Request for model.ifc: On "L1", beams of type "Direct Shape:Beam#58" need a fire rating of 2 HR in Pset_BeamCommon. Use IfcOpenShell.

First a look at what the model holds.

```python
import ifcopenshell
import ifcopenshell.util.element

model = ifcopenshell.open("model.ifc")
print(model.schema)
storey = next(s for s in model.by_type("IfcBuildingStorey") if s.Name == "L1")
beams = [e for e in ifcopenshell.util.element.get_decomposition(storey) if e.is_a("IfcBeam")]
seen = {}
for e in beams:
    element_type = ifcopenshell.util.element.get_type(e)
    key = (element_type.Name if element_type != e and element_type else None, ifcopenshell.util.element.get_pset(e, "Pset_BeamCommon", "FireRating"))
    seen[key] = seen.get(key, 0) + 1
for (name, value), count in sorted(seen.items(), key=str):
    print(count, "x", name, "|", value)
```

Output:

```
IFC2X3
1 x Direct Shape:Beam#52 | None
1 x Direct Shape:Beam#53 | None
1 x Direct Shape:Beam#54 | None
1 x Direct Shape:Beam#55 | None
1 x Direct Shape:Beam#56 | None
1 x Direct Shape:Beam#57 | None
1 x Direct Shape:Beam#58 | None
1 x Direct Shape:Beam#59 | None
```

```python
import ifcopenshell
import ifcopenshell.api.pset
import ifcopenshell.util.element

model = ifcopenshell.open("model.ifc")

storey = next(s for s in model.by_type("IfcBuildingStorey") if s.Name == "L1")
beams = [e for e in ifcopenshell.util.element.get_decomposition(storey) if e.is_a("IfcBeam")]

count = 0
for e in beams:
    element_type = ifcopenshell.util.element.get_type(e)
    if element_type in (None, e) or element_type.Name != "Direct Shape:Beam#58":
        continue
    # add_pset returns the element's existing set when there is one.
    pset = ifcopenshell.api.pset.add_pset(model, product=e, name="Pset_BeamCommon")
    ifcopenshell.api.pset.edit_pset(model, pset=pset, properties={"FireRating": "2 HR"})
    count += 1

print(count, "beams updated")

model.write("model-out.ifc")
```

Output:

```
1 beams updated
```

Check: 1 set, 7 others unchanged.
